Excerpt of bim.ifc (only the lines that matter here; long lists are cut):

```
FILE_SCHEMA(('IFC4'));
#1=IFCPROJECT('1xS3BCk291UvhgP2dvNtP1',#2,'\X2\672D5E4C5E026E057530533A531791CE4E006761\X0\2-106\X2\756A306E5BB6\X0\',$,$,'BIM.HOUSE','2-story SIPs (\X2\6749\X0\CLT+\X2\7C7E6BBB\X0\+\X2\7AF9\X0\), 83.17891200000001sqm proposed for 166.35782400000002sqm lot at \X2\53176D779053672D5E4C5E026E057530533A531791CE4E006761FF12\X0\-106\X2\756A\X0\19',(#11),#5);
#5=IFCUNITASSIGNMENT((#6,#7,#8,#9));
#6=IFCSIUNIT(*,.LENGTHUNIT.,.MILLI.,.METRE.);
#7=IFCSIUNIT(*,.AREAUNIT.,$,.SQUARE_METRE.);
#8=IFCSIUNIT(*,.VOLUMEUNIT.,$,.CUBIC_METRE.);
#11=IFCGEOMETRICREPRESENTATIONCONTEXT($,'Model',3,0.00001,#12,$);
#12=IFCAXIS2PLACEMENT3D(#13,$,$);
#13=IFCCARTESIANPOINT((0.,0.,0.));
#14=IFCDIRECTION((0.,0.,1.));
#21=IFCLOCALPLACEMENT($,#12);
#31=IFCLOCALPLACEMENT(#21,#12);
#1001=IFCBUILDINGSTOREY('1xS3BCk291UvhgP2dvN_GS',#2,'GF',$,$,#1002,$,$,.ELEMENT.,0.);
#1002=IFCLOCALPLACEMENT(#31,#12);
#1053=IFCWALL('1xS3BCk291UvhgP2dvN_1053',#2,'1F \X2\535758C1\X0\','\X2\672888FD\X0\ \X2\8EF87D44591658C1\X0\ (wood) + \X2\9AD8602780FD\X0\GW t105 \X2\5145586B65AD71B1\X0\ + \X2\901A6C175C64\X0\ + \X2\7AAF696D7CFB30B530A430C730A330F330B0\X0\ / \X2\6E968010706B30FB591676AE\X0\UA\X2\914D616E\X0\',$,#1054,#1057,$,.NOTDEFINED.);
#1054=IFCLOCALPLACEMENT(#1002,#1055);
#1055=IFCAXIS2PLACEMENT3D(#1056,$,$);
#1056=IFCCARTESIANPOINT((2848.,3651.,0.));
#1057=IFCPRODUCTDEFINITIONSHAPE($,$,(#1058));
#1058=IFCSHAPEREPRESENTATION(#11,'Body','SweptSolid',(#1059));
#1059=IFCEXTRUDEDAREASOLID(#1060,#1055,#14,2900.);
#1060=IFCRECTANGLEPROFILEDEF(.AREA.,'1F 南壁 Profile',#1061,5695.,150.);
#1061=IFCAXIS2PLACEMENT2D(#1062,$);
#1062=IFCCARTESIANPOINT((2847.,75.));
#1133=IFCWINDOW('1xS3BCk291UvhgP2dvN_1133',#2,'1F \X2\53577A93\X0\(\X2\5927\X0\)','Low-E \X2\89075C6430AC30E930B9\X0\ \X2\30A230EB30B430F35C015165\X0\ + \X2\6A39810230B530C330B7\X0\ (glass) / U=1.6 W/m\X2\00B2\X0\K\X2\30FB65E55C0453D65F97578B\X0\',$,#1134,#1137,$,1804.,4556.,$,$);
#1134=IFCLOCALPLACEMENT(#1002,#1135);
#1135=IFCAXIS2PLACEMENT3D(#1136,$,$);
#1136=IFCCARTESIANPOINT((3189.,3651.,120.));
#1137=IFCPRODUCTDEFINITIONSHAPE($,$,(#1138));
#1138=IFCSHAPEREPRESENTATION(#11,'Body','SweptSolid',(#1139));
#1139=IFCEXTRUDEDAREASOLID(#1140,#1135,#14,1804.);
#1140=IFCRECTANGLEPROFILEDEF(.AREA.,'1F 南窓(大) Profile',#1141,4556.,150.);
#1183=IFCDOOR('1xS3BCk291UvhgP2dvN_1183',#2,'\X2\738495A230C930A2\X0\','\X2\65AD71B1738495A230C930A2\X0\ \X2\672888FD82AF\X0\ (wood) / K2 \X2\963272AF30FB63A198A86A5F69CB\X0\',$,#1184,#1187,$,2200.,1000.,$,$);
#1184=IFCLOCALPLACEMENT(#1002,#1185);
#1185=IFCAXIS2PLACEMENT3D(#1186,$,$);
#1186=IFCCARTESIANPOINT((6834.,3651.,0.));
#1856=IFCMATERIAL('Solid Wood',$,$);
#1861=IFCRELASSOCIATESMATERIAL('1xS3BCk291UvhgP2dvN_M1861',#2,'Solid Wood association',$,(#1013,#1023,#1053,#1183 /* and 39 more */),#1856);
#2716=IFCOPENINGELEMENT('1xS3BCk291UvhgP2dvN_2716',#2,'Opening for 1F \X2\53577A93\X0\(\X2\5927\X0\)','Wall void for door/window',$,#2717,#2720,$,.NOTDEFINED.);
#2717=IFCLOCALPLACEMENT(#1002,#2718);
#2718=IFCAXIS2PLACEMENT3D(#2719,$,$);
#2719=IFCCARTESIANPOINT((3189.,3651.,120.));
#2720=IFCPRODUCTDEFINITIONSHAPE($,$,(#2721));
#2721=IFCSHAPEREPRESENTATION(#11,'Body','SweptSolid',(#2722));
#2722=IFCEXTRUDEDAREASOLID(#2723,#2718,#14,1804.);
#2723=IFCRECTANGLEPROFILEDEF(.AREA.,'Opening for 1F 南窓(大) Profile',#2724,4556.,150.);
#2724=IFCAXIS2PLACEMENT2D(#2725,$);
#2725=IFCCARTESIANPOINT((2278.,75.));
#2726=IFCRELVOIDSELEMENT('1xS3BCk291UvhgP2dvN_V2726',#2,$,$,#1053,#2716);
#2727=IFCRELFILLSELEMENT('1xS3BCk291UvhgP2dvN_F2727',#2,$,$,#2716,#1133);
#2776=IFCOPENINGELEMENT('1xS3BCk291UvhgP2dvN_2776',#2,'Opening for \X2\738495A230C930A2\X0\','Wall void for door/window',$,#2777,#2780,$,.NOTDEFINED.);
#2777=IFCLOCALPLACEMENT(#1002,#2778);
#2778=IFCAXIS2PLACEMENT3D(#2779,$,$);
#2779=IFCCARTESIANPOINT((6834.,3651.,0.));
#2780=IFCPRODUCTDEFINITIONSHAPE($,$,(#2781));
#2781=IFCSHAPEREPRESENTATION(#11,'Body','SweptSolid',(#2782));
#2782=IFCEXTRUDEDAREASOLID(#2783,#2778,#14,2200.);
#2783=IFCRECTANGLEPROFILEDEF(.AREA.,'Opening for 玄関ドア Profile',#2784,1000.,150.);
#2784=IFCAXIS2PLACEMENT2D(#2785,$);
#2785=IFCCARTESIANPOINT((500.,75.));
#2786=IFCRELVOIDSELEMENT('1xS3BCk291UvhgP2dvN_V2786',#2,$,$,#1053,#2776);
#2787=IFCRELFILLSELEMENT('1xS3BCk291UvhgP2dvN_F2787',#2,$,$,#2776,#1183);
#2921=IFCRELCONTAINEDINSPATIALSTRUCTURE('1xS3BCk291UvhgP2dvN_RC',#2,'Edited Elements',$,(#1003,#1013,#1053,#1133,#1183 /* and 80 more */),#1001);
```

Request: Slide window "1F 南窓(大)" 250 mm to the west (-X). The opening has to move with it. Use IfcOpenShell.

```python
import ifcopenshell
import ifcopenshell.api.geometry
import ifcopenshell.util.placement
import ifcopenshell.util.unit

model = ifcopenshell.open("bim.ifc")
unit_scale = ifcopenshell.util.unit.calculate_unit_scale(model)

window = model.by_guid("1xS3BCk291UvhgP2dvN_1133")
opening = window.FillsVoids[0].RelatingOpeningElement
wall = opening.VoidsElements[0].RelatingBuildingElement

wall_matrix = ifcopenshell.util.placement.get_local_placement(wall.ObjectPlacement)
shift = wall_matrix[:3, 0] * -0.25 / unit_scale
before = ifcopenshell.util.placement.get_local_placement(window.ObjectPlacement)[:3, 3].copy()

# The window is not placed relative to its opening, so move both.
for product in (opening, window):
    matrix = ifcopenshell.util.placement.get_local_placement(product.ObjectPlacement)
    matrix[:3, 3] += shift
    ifcopenshell.api.geometry.edit_object_placement(model, product=product, matrix=matrix, is_si=False)

after = ifcopenshell.util.placement.get_local_placement(window.ObjectPlacement)[:3, 3]
print("window moved by", (after - before).round(3) + 0.0)

model.write("bim_updated.ifc")
```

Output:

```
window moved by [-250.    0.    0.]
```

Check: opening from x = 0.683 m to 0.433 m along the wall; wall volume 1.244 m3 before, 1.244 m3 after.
